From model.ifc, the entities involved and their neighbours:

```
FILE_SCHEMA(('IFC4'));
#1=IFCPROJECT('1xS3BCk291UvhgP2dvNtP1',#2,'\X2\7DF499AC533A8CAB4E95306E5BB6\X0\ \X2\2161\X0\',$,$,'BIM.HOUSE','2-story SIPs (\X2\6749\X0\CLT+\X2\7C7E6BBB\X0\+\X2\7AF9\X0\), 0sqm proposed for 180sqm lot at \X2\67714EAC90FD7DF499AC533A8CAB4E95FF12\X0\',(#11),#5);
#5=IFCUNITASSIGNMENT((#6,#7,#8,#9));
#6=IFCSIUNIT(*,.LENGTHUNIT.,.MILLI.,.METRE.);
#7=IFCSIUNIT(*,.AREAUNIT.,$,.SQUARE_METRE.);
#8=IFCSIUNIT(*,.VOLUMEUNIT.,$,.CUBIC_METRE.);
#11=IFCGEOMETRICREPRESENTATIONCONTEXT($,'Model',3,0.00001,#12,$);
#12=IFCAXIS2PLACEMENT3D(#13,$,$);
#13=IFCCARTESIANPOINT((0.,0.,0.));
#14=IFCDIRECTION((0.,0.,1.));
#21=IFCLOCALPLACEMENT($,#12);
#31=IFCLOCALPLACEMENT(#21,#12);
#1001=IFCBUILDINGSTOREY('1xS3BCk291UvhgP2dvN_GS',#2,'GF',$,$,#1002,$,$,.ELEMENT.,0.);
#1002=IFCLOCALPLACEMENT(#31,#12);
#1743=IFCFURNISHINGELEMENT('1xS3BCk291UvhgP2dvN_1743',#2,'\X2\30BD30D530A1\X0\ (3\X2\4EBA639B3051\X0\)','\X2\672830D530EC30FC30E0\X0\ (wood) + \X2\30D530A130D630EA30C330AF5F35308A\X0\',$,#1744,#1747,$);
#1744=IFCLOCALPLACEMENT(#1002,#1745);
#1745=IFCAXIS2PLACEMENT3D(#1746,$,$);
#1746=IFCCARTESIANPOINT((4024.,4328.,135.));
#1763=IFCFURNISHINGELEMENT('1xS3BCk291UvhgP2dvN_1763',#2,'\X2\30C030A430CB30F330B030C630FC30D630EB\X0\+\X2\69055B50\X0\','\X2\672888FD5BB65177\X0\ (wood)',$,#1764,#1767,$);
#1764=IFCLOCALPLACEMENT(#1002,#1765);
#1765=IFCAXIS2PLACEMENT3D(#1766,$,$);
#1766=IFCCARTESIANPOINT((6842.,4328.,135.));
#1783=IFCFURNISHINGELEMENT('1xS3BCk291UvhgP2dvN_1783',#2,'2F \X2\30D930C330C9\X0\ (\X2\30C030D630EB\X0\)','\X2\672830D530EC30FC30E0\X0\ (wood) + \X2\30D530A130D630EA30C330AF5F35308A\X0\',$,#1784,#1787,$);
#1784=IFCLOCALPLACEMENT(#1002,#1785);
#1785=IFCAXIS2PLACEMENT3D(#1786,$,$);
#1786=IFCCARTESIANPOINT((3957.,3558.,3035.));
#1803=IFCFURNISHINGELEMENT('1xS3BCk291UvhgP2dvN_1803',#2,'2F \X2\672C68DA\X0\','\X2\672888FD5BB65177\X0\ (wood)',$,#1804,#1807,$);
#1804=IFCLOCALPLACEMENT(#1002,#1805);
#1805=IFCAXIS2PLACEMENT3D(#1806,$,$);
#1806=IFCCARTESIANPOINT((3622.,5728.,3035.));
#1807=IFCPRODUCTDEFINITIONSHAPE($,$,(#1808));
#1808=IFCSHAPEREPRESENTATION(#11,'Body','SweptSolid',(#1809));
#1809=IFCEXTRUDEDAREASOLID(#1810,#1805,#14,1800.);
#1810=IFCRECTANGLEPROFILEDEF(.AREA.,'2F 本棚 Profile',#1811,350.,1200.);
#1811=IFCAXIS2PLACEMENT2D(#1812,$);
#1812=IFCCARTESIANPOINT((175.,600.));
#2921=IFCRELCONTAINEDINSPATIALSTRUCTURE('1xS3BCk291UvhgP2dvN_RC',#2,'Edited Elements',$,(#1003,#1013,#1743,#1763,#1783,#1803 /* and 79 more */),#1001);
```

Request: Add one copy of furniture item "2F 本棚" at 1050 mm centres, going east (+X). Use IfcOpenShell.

```python
import numpy as np
import ifcopenshell
import ifcopenshell.api.geometry
import ifcopenshell.api.root
import ifcopenshell.util.element
import ifcopenshell.util.placement

model = ifcopenshell.open("model.ifc")


def reuse_history(source, copy):
    """copy_class also copies each property set's owner history, people and application; keep the originals."""
    for rel in copy.IsDefinedBy:
        if rel.is_a("IfcRelDefinesByProperties") and (history := rel.RelatingPropertyDefinition.OwnerHistory):
            rel.RelatingPropertyDefinition.OwnerHistory = source.OwnerHistory
            ifcopenshell.util.element.remove_deep2(model, history)


source = model.by_guid("1xS3BCk291UvhgP2dvN_1803")
base = ifcopenshell.util.placement.get_local_placement(source.ObjectPlacement)
step = np.array([1.0, 0.0, 0.0]) * 1050.0

for i in range(1, 2):
    copy = ifcopenshell.api.root.copy_class(model, product=source)
    copy.Representation = ifcopenshell.util.element.copy_deep(
        model, source.Representation, exclude=["IfcGeometricRepresentationContext", "IfcRepresentationMap"]
    )
    reuse_history(source, copy)
    matrix = base.copy()
    matrix[:3, 3] += i * step
    print("added at", matrix[:3, 3].round(3) + 0.0)
    ifcopenshell.api.geometry.edit_object_placement(model, product=copy, matrix=matrix, is_si=False)

model.write("model_v2.ifc")
```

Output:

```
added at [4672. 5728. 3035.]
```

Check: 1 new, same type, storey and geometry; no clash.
